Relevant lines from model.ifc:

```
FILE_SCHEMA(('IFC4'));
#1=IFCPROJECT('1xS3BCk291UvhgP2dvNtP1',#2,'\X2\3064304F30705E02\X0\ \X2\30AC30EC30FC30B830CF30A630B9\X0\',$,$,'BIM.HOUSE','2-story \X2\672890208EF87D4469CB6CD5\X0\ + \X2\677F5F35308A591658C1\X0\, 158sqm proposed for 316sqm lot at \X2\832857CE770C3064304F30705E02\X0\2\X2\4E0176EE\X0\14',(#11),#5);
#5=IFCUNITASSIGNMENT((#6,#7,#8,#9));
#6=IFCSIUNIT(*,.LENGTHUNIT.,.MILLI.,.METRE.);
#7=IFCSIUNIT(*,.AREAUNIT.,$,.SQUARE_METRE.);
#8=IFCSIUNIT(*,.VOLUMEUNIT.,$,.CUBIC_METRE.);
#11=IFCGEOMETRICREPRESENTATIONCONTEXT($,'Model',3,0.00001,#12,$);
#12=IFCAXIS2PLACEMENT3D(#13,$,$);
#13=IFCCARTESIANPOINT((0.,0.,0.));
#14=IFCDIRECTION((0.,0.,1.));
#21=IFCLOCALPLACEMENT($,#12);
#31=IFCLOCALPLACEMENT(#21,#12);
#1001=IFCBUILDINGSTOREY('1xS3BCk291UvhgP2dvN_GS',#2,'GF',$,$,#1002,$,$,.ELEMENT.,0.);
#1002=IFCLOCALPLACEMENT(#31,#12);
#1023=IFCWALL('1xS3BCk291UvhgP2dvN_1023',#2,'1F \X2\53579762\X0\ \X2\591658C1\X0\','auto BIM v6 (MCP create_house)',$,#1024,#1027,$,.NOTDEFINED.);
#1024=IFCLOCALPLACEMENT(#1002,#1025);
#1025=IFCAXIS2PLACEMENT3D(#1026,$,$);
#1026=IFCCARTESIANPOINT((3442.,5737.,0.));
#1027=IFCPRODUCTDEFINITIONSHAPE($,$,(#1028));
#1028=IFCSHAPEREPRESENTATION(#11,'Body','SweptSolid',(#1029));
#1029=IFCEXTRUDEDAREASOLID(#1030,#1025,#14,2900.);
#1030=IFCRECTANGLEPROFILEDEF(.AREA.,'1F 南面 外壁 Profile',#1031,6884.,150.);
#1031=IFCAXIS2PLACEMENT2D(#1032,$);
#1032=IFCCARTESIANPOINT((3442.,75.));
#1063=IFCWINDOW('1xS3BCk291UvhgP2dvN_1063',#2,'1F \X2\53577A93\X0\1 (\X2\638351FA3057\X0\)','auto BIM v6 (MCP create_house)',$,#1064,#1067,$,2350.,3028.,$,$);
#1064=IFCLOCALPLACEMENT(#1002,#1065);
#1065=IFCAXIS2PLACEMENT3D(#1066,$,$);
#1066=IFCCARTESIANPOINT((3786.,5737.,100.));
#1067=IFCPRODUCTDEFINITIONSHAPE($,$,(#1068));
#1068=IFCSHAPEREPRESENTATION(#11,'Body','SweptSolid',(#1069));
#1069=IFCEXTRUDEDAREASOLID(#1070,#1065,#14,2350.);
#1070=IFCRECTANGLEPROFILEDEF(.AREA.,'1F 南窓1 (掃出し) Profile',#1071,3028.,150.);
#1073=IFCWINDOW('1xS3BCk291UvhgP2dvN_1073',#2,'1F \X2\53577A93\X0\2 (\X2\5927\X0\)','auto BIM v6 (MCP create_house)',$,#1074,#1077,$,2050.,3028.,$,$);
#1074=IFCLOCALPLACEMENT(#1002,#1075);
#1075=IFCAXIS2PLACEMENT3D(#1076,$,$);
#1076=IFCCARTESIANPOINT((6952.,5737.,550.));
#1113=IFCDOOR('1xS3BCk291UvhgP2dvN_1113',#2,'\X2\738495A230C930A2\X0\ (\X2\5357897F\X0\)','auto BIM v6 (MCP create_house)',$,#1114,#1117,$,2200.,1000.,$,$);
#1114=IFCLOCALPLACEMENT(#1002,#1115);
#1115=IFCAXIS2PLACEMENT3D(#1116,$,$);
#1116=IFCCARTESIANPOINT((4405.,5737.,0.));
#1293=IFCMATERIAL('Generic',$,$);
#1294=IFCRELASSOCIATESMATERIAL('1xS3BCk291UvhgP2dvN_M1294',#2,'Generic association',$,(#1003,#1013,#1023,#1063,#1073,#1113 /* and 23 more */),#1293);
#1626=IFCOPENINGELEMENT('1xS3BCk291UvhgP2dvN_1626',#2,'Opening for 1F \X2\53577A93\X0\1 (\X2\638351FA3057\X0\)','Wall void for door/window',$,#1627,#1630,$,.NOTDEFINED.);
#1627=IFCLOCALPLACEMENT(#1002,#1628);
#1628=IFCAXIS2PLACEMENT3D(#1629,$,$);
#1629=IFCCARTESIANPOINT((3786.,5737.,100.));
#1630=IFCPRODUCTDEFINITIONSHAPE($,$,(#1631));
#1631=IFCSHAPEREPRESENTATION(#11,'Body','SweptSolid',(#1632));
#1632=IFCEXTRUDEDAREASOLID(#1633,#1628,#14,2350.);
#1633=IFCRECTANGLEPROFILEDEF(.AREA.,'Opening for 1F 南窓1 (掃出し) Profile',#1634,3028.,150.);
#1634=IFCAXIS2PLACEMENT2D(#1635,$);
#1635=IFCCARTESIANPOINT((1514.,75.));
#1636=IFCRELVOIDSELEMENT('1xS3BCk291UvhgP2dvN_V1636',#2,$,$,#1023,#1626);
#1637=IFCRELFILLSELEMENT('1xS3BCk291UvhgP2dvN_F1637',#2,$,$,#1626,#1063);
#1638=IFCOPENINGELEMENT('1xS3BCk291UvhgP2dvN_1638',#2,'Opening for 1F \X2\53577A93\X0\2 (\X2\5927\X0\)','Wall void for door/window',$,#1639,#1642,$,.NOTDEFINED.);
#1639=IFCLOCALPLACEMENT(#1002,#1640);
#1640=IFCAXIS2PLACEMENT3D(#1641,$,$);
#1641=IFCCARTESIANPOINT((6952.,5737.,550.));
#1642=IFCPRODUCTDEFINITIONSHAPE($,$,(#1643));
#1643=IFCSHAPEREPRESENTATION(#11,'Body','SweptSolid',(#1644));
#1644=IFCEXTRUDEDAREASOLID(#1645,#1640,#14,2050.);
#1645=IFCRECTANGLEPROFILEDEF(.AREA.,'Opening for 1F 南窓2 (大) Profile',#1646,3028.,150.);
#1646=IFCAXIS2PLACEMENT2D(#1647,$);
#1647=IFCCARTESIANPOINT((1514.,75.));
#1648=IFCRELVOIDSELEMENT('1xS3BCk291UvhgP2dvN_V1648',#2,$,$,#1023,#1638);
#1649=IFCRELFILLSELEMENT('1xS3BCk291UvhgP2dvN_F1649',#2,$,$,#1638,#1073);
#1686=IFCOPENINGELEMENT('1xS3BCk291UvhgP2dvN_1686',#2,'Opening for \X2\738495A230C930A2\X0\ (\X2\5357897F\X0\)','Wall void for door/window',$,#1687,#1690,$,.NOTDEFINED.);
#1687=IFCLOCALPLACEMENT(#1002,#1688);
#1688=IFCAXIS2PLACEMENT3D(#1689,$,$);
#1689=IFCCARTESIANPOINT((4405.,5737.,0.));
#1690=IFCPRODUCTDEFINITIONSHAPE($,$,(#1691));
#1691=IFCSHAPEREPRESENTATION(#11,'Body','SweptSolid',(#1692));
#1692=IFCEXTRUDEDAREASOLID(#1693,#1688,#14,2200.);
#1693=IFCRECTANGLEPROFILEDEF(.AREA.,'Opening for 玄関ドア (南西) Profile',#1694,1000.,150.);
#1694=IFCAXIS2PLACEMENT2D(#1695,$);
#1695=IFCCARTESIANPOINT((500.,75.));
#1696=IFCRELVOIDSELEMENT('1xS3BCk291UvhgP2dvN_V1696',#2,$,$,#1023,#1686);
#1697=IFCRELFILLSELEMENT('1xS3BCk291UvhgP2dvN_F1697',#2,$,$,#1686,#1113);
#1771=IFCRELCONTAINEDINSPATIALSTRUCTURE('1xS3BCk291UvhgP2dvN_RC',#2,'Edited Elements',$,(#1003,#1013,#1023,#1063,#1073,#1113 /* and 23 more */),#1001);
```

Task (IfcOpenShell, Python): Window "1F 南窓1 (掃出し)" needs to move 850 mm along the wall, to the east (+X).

```python
import ifcopenshell
import ifcopenshell.api.geometry
import ifcopenshell.util.placement

model = ifcopenshell.open("model.ifc")

window = model.by_id(1063)
opening = window.FillsVoids[0].RelatingOpeningElement
wall = opening.VoidsElements[0].RelatingBuildingElement

wall_matrix = ifcopenshell.util.placement.get_local_placement(wall.ObjectPlacement)
shift = wall_matrix[:3, 0] * 850.0
before = ifcopenshell.util.placement.get_local_placement(window.ObjectPlacement)[:3, 3].copy()

# The window is not placed relative to its opening, so move both.
for product in (opening, window):
    matrix = ifcopenshell.util.placement.get_local_placement(product.ObjectPlacement)
    matrix[:3, 3] += shift
    ifcopenshell.api.geometry.edit_object_placement(model, product=product, matrix=matrix, is_si=False)

after = ifcopenshell.util.placement.get_local_placement(window.ObjectPlacement)[:3, 3]
print("window moved by", (after - before).round(3) + 0.0)

model.write("model_rev.ifc")
```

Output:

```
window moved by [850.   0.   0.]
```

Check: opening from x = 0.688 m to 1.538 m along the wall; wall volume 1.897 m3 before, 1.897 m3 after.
